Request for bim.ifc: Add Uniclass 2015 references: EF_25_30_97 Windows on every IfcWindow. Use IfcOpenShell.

First a look at what the model holds.

```python
import ifcopenshell

model = ifcopenshell.open("bim.ifc")
print(model.schema)
print("classifications:", [c.Name for c in model.by_type("IfcClassification")])
for ifc_class in ("IfcDoor", "IfcRoof", "IfcStair", "IfcWall", "IfcWindow"):
    print(ifc_class, len(model.by_type(ifc_class)))
```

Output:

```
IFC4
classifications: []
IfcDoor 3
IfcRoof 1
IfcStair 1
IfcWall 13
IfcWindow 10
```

```python
import ifcopenshell
import ifcopenshell.api.classification

model = ifcopenshell.open("bim.ifc")

system = ifcopenshell.api.classification.add_classification(model, classification="Uniclass 2015")

codes = {
    "IfcWindow": ("EF_25_30_97", "Windows"),
}
for ifc_class, (code, name) in codes.items():
    products = model.by_type(ifc_class)
    ifcopenshell.api.classification.add_reference(
        model, products=products, classification=system, identification=code, name=name
    )
    print(code, len(products))

model.write("bim_updated.ifc")
```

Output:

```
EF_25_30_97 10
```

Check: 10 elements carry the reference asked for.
